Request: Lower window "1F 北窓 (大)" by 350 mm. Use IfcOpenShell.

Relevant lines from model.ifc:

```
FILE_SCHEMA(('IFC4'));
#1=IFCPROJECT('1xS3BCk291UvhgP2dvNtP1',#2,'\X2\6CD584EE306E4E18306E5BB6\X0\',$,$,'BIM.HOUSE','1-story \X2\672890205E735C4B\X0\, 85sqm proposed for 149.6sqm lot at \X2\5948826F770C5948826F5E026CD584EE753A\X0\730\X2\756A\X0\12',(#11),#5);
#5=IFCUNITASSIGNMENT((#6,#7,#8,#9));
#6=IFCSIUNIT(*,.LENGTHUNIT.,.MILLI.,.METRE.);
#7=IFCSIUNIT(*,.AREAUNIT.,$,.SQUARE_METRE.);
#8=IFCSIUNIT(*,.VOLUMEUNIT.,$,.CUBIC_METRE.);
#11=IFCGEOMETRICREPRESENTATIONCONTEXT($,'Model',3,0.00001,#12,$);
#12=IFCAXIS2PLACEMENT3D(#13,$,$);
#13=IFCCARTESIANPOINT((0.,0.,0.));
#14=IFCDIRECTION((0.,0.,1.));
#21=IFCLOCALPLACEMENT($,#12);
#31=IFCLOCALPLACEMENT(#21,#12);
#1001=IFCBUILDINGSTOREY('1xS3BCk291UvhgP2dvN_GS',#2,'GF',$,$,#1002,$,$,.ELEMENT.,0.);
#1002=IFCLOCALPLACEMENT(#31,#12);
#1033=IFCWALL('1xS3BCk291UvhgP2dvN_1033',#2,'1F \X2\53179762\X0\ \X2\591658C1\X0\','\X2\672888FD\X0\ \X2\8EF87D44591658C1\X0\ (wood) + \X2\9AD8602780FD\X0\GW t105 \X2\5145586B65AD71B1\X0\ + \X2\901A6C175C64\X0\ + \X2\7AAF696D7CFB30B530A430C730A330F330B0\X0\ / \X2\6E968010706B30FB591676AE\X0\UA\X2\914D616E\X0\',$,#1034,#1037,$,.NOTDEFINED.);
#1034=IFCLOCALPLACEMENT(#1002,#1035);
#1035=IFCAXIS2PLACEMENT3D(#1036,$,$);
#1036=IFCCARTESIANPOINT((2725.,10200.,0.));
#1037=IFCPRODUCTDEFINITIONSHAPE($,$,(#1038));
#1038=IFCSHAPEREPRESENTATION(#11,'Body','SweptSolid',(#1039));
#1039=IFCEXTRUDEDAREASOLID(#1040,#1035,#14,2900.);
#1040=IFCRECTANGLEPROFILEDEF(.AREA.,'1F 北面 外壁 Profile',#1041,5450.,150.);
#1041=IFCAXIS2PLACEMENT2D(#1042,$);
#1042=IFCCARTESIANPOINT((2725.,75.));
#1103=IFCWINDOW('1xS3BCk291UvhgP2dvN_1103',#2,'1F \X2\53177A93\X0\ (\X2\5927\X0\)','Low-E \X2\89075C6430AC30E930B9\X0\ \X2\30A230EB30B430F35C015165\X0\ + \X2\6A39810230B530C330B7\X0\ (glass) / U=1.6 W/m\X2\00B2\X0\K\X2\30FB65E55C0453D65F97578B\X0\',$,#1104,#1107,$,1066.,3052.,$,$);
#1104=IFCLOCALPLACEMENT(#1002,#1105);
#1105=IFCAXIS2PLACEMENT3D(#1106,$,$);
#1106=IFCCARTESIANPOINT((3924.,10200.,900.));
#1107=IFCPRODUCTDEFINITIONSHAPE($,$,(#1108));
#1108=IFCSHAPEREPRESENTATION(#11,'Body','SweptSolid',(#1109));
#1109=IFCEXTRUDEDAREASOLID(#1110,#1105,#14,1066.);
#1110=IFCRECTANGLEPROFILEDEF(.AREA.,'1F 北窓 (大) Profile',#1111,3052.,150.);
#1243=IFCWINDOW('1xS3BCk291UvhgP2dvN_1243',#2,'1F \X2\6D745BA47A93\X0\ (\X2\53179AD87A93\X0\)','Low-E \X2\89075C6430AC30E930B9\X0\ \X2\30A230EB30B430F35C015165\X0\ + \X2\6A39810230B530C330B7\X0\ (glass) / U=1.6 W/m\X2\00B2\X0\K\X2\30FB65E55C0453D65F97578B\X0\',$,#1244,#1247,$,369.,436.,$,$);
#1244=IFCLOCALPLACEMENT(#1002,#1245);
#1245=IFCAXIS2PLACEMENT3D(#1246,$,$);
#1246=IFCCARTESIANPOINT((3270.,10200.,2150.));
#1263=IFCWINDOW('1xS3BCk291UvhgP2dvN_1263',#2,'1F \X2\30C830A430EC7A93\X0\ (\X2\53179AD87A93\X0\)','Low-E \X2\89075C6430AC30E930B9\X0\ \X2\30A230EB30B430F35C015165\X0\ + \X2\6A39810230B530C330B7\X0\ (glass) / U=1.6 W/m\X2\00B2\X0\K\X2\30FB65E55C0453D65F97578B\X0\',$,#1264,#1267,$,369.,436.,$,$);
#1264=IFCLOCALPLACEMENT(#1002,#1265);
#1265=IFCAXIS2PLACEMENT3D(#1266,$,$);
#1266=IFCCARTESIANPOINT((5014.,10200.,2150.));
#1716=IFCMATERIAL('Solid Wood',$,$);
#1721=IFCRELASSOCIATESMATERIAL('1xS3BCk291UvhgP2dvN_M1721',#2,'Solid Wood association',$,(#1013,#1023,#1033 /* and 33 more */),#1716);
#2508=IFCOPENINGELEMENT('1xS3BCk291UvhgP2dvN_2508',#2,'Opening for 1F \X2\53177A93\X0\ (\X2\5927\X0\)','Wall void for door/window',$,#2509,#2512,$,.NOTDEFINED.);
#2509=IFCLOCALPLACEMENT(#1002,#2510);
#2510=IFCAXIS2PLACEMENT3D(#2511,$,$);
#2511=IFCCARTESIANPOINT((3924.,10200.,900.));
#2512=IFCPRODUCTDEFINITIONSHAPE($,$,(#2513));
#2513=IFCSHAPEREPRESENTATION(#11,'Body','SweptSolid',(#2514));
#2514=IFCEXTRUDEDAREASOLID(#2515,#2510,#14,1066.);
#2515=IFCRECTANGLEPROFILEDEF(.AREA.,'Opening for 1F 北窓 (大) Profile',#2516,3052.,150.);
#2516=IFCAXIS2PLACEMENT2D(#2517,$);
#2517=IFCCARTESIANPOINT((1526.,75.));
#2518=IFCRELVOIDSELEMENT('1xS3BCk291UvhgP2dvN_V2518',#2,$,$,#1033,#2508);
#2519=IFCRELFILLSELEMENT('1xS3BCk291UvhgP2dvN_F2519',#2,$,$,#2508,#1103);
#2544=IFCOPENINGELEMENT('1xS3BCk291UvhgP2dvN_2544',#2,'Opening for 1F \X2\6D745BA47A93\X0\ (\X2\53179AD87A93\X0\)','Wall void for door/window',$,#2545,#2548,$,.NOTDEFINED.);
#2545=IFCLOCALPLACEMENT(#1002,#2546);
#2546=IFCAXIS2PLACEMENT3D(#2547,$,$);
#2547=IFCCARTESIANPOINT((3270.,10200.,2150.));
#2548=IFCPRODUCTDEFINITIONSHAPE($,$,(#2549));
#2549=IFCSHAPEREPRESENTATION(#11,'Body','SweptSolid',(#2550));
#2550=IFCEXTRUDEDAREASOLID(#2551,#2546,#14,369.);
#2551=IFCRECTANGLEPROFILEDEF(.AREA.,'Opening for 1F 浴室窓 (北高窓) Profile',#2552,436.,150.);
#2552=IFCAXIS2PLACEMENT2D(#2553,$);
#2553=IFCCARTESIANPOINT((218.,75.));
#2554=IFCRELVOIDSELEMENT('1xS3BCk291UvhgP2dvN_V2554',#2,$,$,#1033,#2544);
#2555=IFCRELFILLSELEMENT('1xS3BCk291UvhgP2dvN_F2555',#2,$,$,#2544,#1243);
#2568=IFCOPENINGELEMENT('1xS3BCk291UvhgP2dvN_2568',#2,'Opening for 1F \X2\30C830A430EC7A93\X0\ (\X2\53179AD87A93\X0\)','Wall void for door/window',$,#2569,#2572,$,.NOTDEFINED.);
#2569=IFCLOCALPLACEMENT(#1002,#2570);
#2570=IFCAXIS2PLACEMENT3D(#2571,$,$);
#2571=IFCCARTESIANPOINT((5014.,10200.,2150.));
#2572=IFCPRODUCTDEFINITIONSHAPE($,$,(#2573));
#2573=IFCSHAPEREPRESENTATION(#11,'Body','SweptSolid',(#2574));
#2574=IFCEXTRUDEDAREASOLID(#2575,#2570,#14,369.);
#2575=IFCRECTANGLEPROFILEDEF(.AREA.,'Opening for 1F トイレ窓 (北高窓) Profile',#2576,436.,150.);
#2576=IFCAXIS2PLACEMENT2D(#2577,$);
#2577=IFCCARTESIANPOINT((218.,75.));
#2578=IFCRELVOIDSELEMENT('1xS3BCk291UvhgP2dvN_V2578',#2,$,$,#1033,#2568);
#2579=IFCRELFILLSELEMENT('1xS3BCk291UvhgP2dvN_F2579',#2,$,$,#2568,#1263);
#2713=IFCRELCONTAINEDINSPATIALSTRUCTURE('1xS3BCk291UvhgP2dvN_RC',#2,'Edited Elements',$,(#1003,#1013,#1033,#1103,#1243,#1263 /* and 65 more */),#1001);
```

```python
import numpy as np
import ifcopenshell
import ifcopenshell.api.geometry
import ifcopenshell.util.placement
import ifcopenshell.util.unit

model = ifcopenshell.open("model.ifc")
unit_scale = ifcopenshell.util.unit.calculate_unit_scale(model)

window = model.by_guid("1xS3BCk291UvhgP2dvN_1103")
opening = window.FillsVoids[0].RelatingOpeningElement
dz = -0.35 / unit_scale

shift = np.array([0.0, 0.0, dz])
# The window is not placed relative to its opening, so move both.
for product in (opening, window):
    matrix = ifcopenshell.util.placement.get_local_placement(product.ObjectPlacement)
    matrix[:3, 3] += shift
    ifcopenshell.api.geometry.edit_object_placement(model, product=product, matrix=matrix, is_si=False)

print(f"moved by {dz * unit_scale:+.3f} m")

model.write("model-out.ifc")
```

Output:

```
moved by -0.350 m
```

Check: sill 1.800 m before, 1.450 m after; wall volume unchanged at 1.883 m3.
